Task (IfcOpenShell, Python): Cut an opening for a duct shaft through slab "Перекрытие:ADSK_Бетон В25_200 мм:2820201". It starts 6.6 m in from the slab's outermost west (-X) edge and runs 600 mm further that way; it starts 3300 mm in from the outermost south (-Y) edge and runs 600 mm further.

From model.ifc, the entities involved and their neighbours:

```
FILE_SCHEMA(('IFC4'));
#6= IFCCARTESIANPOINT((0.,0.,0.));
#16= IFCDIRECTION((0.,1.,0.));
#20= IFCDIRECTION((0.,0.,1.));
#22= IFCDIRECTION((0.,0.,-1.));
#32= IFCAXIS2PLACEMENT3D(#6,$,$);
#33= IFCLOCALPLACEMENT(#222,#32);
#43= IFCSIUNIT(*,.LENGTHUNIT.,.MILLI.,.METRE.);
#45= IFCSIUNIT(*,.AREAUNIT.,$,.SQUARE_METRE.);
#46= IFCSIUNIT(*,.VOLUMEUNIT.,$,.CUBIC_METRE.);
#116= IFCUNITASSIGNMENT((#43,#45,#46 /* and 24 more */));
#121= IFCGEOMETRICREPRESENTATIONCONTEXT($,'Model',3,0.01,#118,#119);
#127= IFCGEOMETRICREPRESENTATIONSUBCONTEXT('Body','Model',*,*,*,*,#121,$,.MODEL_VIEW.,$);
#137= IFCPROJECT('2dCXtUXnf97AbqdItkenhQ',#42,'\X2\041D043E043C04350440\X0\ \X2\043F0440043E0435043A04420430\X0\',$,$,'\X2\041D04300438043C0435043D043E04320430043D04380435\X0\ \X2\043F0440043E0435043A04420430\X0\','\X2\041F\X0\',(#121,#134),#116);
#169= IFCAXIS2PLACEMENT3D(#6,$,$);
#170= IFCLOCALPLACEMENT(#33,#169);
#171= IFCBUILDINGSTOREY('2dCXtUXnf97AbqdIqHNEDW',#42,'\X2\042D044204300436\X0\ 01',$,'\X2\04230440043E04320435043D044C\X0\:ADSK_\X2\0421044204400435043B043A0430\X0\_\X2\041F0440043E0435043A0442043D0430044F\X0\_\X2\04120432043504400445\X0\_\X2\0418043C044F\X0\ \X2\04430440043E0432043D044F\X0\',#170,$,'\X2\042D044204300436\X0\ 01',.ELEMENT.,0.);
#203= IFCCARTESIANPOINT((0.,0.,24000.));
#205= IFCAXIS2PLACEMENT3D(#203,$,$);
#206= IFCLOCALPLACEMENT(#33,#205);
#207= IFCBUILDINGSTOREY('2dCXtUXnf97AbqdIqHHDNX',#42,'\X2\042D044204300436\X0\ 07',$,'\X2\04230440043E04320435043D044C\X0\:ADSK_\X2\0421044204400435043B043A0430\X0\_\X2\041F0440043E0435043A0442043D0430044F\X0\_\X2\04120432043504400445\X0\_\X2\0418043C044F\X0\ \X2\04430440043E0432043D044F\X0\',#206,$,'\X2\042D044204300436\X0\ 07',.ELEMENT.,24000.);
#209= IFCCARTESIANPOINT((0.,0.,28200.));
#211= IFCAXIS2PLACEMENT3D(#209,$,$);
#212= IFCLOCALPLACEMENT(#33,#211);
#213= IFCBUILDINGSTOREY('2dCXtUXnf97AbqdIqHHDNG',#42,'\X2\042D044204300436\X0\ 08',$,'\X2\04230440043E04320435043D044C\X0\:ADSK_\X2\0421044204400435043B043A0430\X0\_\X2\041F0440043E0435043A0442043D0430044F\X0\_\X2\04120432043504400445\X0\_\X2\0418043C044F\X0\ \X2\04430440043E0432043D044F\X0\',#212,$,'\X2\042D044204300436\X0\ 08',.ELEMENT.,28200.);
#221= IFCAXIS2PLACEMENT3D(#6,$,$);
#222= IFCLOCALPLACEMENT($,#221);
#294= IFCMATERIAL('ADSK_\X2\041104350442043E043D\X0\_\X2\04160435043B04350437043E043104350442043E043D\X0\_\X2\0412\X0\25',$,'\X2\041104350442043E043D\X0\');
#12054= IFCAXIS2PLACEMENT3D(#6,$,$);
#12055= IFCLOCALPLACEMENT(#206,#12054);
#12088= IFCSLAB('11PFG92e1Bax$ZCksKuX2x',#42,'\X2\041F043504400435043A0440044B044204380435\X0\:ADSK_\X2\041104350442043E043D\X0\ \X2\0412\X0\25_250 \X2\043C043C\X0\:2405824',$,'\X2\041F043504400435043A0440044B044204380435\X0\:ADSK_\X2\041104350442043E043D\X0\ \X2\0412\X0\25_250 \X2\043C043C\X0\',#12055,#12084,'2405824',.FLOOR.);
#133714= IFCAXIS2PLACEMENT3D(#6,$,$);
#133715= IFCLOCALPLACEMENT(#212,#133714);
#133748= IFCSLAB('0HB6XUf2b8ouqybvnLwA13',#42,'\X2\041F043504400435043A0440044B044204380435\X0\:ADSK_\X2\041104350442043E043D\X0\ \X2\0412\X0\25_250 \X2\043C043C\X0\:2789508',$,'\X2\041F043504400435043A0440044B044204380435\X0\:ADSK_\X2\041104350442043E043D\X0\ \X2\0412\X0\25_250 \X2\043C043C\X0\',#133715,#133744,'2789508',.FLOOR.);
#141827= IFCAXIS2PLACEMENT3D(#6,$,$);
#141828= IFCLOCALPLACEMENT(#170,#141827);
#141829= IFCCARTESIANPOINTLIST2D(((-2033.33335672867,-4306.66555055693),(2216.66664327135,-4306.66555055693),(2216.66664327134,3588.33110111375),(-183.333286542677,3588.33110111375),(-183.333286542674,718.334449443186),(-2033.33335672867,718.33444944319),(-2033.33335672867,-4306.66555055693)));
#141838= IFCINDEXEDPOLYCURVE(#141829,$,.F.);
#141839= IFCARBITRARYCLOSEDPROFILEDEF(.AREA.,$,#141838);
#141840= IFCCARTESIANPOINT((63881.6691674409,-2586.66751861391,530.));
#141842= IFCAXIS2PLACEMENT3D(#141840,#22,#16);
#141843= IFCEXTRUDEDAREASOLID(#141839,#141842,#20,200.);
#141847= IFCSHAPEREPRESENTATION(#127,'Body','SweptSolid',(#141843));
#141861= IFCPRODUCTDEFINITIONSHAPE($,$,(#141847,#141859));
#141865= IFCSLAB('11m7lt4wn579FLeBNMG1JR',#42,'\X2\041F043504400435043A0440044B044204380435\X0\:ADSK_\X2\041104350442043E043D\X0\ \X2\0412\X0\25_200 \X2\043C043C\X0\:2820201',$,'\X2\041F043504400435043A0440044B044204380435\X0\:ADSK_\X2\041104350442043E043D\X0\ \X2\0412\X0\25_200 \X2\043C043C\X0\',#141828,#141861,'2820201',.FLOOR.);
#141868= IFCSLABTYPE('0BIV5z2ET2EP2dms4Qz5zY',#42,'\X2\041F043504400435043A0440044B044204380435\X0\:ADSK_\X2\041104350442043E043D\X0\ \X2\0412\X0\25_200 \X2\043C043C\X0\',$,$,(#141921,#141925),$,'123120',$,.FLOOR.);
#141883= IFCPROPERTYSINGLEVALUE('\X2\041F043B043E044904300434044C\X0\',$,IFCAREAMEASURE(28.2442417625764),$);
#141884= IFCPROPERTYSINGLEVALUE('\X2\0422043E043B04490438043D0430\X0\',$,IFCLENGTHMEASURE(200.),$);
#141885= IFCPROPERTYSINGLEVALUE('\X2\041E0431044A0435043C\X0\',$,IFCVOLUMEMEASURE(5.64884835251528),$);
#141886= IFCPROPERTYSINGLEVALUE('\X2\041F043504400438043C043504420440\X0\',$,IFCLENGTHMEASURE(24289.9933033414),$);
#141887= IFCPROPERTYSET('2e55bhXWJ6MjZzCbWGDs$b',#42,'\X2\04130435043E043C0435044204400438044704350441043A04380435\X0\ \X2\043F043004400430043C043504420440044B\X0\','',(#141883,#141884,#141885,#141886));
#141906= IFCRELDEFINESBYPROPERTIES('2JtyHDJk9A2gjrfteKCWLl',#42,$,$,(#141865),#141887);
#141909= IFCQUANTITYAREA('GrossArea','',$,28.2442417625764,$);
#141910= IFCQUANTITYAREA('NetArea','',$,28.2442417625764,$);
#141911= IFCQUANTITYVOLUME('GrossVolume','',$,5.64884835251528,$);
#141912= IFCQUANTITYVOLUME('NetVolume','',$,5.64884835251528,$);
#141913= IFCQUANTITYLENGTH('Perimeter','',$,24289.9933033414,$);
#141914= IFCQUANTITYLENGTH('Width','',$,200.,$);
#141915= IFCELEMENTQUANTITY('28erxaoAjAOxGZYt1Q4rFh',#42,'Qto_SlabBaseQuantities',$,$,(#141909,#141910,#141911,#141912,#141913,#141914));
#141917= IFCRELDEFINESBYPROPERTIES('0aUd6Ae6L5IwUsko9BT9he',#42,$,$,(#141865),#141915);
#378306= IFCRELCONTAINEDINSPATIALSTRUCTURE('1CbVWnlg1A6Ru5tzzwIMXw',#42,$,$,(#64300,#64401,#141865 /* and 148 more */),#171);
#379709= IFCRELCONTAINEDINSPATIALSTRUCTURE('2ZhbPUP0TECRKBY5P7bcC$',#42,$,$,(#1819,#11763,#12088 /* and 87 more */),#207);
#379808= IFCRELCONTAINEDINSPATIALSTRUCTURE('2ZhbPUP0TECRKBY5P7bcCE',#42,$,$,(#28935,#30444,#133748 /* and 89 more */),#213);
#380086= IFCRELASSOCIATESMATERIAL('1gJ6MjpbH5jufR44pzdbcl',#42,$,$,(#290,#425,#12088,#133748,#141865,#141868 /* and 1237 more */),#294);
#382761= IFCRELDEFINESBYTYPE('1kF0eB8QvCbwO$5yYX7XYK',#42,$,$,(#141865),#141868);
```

```python
import numpy as np
import ifcopenshell
import ifcopenshell.api.feature
import ifcopenshell.api.geometry
import ifcopenshell.api.pset
import ifcopenshell.api.root
import ifcopenshell.geom
import ifcopenshell.util.element
import ifcopenshell.util.placement
import ifcopenshell.util.representation
import ifcopenshell.util.shape
import ifcopenshell.util.unit

model = ifcopenshell.open("model.ifc")
unit_scale = ifcopenshell.util.unit.calculate_unit_scale(model)
area_scale = ifcopenshell.util.unit.calculate_unit_scale(model, "AREAUNIT")
volume_scale = ifcopenshell.util.unit.calculate_unit_scale(model, "VOLUMEUNIT")
settings = ifcopenshell.geom.settings()


def volume(element):
    """Net volume in cubic metres, openings subtracted."""
    shape = ifcopenshell.geom.create_shape(settings, element)
    return ifcopenshell.util.shape.get_volume(shape.geometry)


slab = model.by_guid("11m7lt4wn579FLeBNMG1JR")
before = volume(slab)

# Extent in the slab's own axes, in metres. The edges named are its -X and -Y sides.
slab_shape = ifcopenshell.geom.create_shape(settings, slab)
vertices = ifcopenshell.util.shape.get_vertices(slab_shape.geometry)
x_min, y_min, bottom = vertices.min(axis=0)
top = vertices[:, 2].max()

opening = ifcopenshell.api.root.create_entity(model, ifc_class="IfcOpeningElement", name="Duct shaft opening", predefined_type="OPENING")
context = ifcopenshell.util.representation.get_context(model, "Model", "Body", "MODEL_VIEW")
width, depth = 0.6, 0.6
outline = [(0.0, 0.0), (width, 0.0), (width, depth), (0.0, depth), (0.0, 0.0)]
# Overshoot both faces by 50 mm so the cut is clean.
shape = ifcopenshell.api.geometry.add_slab_representation(
    model, context=context, depth=top - bottom + 0.1, polyline=outline
)
ifcopenshell.api.geometry.assign_representation(model, product=opening, representation=shape)

matrix = ifcopenshell.util.placement.get_local_placement(slab.ObjectPlacement)
matrix[:, 3] = matrix @ np.append(np.array([x_min + 6.6, y_min + 3.3, bottom - 0.05]) / unit_scale, 1.0)
ifcopenshell.api.geometry.edit_object_placement(model, product=opening, matrix=matrix, is_si=False)
ifcopenshell.api.feature.add_feature(model, feature=opening, element=slab)

after = volume(slab)

# Update the slab's stored quantities.
pset = model.by_id(ifcopenshell.util.element.get_pset(slab, "Геометрические параметры", should_inherit=False)["id"])
ifcopenshell.api.pset.edit_pset(model, pset=pset, properties={
    "Площадь": model.create_entity("IfcAreaMeasure", after / (top - bottom) / area_scale),
    "Объем": model.create_entity("IfcVolumeMeasure", after / volume_scale),
})
qto = model.by_id(ifcopenshell.util.element.get_pset(slab, "Qto_SlabBaseQuantities", should_inherit=False)["id"])
ifcopenshell.api.pset.edit_qto(model, qto=qto, properties={
    "NetArea": after / (top - bottom) / area_scale,
    "NetVolume": after / volume_scale,
})

print(f"slab volume {before:.3f} -> {after:.3f} m3")

model.write("model_v2.ifc")
```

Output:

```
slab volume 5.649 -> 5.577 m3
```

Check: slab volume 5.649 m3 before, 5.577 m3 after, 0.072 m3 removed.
